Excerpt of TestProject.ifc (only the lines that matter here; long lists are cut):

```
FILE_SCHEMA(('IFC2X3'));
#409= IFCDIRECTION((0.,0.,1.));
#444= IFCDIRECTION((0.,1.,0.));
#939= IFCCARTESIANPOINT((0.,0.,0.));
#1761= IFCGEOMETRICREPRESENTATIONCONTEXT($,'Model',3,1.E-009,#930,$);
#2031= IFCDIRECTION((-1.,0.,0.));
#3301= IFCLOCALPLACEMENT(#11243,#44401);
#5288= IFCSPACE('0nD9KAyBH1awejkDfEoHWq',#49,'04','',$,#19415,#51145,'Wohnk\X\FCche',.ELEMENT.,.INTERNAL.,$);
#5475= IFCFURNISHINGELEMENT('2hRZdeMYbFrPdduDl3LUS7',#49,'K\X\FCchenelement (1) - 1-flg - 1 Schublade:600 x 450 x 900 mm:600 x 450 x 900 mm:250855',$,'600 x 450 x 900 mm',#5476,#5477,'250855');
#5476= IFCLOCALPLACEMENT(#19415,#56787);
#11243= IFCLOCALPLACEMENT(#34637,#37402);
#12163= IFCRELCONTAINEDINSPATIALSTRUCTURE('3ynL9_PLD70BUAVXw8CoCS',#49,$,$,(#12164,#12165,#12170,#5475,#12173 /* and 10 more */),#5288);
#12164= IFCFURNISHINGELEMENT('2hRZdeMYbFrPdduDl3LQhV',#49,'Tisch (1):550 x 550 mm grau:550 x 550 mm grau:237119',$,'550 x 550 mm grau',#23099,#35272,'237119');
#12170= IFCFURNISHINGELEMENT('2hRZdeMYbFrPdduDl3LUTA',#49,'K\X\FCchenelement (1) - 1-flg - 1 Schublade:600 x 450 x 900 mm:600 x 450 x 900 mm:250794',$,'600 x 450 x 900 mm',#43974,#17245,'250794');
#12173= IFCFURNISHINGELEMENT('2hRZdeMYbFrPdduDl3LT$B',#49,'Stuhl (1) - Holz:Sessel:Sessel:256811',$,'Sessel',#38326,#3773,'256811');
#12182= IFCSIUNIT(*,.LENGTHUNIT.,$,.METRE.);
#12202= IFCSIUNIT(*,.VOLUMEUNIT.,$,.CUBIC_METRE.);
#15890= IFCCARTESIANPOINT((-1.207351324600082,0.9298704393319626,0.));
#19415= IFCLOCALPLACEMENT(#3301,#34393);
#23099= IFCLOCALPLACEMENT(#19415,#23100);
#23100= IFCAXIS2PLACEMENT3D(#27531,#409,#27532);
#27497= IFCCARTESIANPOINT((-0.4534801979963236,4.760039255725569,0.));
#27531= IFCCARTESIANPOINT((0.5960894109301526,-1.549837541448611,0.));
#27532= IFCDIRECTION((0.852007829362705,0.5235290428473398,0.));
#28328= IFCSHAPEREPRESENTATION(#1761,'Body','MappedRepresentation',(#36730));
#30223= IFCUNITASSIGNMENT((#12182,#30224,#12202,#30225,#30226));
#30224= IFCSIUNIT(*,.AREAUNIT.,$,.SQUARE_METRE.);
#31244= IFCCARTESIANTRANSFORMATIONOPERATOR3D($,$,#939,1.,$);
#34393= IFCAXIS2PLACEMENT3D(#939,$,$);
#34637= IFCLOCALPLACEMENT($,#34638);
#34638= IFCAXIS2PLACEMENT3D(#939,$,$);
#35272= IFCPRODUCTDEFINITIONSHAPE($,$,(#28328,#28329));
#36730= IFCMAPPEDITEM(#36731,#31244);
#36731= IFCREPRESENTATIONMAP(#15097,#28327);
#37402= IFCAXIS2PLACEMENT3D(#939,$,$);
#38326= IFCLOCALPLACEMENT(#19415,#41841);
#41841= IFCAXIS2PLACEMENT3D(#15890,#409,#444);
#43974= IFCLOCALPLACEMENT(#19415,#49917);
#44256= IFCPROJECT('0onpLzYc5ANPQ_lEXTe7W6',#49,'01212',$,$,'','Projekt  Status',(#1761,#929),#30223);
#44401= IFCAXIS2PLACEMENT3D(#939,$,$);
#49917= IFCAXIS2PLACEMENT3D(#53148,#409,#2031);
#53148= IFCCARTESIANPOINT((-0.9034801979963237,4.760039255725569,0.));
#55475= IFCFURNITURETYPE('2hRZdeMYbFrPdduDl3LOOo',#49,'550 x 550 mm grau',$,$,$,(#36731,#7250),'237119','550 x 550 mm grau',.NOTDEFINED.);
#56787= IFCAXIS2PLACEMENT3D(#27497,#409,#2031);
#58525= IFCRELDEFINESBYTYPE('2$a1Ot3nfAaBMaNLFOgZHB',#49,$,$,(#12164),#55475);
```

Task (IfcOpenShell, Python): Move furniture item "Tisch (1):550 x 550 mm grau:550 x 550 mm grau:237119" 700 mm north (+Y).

```python
import ifcopenshell
import ifcopenshell.api.geometry
import ifcopenshell.util.placement

model = ifcopenshell.open("TestProject.ifc")

item = model.by_guid("2hRZdeMYbFrPdduDl3LQhV")
matrix = ifcopenshell.util.placement.get_local_placement(item.ObjectPlacement)
matrix[1, 3] += 0.7
ifcopenshell.api.geometry.edit_object_placement(model, product=item, matrix=matrix, is_si=False)

print(ifcopenshell.util.placement.get_local_placement(item.ObjectPlacement).round(3) + 0.0)

model.write("TestProject_rev.ifc")
```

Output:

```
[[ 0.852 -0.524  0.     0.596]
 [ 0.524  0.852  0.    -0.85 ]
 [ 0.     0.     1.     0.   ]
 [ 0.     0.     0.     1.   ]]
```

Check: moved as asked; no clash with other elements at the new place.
